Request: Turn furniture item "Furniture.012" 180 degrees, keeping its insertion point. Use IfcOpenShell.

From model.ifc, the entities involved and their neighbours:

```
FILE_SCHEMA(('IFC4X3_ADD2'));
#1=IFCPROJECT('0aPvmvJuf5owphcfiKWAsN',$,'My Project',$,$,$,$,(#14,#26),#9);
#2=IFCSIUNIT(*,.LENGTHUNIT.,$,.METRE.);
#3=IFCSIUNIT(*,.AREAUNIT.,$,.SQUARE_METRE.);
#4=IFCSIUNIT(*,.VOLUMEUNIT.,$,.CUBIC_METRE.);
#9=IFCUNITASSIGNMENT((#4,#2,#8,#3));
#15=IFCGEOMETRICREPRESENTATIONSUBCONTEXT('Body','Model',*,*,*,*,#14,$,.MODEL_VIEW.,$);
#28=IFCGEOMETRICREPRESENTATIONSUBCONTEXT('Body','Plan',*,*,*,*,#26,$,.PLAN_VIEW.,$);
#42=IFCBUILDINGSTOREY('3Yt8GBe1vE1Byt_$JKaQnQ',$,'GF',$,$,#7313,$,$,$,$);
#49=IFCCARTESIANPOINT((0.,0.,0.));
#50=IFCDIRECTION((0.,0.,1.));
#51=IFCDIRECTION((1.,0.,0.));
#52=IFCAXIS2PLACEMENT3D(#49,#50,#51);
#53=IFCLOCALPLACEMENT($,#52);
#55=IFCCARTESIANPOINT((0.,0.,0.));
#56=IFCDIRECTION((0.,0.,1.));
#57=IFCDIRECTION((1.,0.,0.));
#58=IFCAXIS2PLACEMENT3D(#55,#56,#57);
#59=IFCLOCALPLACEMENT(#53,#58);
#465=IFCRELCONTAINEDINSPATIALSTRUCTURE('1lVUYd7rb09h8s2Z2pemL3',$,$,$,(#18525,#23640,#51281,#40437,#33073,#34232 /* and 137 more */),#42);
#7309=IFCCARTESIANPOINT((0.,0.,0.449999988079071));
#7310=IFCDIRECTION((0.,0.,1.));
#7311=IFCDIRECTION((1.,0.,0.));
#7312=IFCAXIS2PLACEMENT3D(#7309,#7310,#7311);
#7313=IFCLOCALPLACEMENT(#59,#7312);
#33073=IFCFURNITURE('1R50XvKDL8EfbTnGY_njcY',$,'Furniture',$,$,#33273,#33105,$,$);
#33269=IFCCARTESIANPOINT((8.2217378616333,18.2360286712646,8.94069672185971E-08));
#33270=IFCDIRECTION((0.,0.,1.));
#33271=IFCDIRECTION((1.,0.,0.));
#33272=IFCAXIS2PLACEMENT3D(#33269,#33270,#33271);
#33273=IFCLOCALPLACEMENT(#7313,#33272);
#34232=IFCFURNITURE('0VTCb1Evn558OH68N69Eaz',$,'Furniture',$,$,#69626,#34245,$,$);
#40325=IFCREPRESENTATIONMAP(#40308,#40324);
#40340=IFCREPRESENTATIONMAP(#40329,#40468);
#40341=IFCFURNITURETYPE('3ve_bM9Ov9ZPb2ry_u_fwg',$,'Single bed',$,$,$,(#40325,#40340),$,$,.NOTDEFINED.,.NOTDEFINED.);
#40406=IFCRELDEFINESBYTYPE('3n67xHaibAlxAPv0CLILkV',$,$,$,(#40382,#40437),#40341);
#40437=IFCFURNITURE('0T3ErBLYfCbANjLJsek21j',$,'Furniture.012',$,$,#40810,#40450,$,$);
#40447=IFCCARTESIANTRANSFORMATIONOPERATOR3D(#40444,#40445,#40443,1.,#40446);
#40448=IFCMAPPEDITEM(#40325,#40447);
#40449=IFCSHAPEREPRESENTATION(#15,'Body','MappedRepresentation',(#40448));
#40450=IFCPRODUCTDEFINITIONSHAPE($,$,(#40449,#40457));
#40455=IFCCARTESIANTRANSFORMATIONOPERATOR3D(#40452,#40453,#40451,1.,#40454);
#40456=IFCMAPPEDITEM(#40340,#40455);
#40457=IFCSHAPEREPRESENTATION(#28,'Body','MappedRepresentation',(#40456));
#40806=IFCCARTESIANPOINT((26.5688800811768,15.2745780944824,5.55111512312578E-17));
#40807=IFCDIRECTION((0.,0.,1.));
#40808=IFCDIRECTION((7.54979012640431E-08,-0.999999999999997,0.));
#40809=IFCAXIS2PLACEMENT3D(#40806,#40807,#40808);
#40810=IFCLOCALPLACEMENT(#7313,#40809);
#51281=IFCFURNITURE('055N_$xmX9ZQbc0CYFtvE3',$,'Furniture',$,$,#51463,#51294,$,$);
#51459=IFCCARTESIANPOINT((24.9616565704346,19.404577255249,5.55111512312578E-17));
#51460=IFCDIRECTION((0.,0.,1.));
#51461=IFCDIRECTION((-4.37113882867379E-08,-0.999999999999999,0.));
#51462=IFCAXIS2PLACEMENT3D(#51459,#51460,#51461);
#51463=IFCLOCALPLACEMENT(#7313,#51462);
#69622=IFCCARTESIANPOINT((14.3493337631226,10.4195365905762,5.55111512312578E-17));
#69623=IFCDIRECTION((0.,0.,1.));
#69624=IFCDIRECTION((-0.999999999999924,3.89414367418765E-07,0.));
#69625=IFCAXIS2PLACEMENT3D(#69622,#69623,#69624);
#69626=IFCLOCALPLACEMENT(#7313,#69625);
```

```python
import ifcopenshell
import ifcopenshell.api.geometry
import ifcopenshell.util.placement

model = ifcopenshell.open("model.ifc")

item = model.by_guid("0T3ErBLYfCbANjLJsek21j")
matrix = ifcopenshell.util.placement.get_local_placement(item.ObjectPlacement)
matrix = matrix @ ifcopenshell.util.placement.rotation(180, "Z")
ifcopenshell.api.geometry.edit_object_placement(model, product=item, matrix=matrix, is_si=False)

print(ifcopenshell.util.placement.get_local_placement(item.ObjectPlacement).round(3) + 0.0)

model.write("model_v2.ifc")
```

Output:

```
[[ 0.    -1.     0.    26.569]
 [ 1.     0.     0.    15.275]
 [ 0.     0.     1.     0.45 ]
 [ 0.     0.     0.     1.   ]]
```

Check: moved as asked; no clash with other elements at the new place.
